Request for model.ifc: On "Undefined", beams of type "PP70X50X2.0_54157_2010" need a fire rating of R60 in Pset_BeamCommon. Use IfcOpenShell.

First a look at what the model holds.

```python
import ifcopenshell
import ifcopenshell.util.element

model = ifcopenshell.open("model.ifc")
print(model.schema)
storey = next(s for s in model.by_type("IfcBuildingStorey") if s.Name == "Undefined")
beams = [e for e in ifcopenshell.util.element.get_decomposition(storey) if e.is_a("IfcBeam")]
seen = {}
for e in beams:
    element_type = ifcopenshell.util.element.get_type(e)
    key = (element_type.Name if element_type != e and element_type else None, ifcopenshell.util.element.get_pset(e, "Pset_BeamCommon", "FireRating"))
    seen[key] = seen.get(key, 0) + 1
for (name, value), count in sorted(seen.items(), key=str):
    print(count, "x", name, "|", value)
```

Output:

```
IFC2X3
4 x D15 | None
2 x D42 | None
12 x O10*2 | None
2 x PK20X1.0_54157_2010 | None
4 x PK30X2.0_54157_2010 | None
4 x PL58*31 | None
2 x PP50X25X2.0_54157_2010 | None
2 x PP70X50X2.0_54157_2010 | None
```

```python
import ifcopenshell
import ifcopenshell.api.pset
import ifcopenshell.util.element

model = ifcopenshell.open("model.ifc")

storey = next(s for s in model.by_type("IfcBuildingStorey") if s.Name == "Undefined")
beams = [e for e in ifcopenshell.util.element.get_decomposition(storey) if e.is_a("IfcBeam")]

count = 0
for e in beams:
    element_type = ifcopenshell.util.element.get_type(e)
    if element_type in (None, e) or element_type.Name != "PP70X50X2.0_54157_2010":
        continue
    found = ifcopenshell.util.element.get_pset(e, "Pset_BeamCommon", should_inherit=False)
    if found:
        pset = model.by_id(found["id"])
        if len(ifcopenshell.util.element.get_elements_by_pset(pset)) > 1:
            pset = ifcopenshell.api.pset.unshare_pset(model, products=[e], pset=pset)[0]
    else:
        pset = ifcopenshell.api.pset.add_pset(model, product=e, name="Pset_BeamCommon")
    ifcopenshell.api.pset.edit_pset(model, pset=pset, properties={"FireRating": "R60"})
    count += 1

print(count, "beams updated")

model.write("model_updated.ifc")
```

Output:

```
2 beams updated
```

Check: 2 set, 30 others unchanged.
